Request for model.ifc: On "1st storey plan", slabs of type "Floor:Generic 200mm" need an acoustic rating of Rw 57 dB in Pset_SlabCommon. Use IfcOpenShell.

First a look at what the model holds.

```python
import ifcopenshell
import ifcopenshell.util.element

model = ifcopenshell.open("model.ifc")
print(model.schema)
storey = next(s for s in model.by_type("IfcBuildingStorey") if s.Name == "1st storey plan")
slabs = [e for e in ifcopenshell.util.element.get_decomposition(storey) if e.is_a("IfcSlab")]
seen = {}
for e in slabs:
    element_type = ifcopenshell.util.element.get_type(e)
    key = (element_type.Name if element_type != e and element_type else None, ifcopenshell.util.element.get_pset(e, "Pset_SlabCommon", "AcousticRating"))
    seen[key] = seen.get(key, 0) + 1
for (name, value), count in sorted(seen.items(), key=str):
    print(count, "x", name, "|", value)
```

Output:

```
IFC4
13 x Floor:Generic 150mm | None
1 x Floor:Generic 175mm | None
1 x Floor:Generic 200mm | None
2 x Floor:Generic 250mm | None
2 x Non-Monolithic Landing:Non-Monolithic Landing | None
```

```python
import ifcopenshell
import ifcopenshell.api.pset
import ifcopenshell.util.element

model = ifcopenshell.open("model.ifc")

storey = next(s for s in model.by_type("IfcBuildingStorey") if s.Name == "1st storey plan")
slabs = [e for e in ifcopenshell.util.element.get_decomposition(storey) if e.is_a("IfcSlab")]

count = 0
for e in slabs:
    element_type = ifcopenshell.util.element.get_type(e)
    if element_type in (None, e) or element_type.Name != "Floor:Generic 200mm":
        continue
    # add_pset returns the element's existing set when there is one.
    pset = ifcopenshell.api.pset.add_pset(model, product=e, name="Pset_SlabCommon")
    ifcopenshell.api.pset.edit_pset(model, pset=pset, properties={"AcousticRating": "Rw 57 dB"})
    count += 1

print(count, "slabs updated")

model.write("model_v2.ifc")
```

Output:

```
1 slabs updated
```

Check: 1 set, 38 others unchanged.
